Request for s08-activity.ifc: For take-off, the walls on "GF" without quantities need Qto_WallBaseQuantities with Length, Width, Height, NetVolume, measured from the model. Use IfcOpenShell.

First a look at what the model holds.

```python
import ifcopenshell
import ifcopenshell.util.element
import ifcopenshell.util.unit

model = ifcopenshell.open("s08-activity.ifc")
print(model.schema)
for unit_type in ("LENGTHUNIT", "AREAUNIT", "VOLUMEUNIT"):
    print(unit_type, ifcopenshell.util.unit.calculate_unit_scale(model, unit_type))
storey = next(s for s in model.by_type("IfcBuildingStorey") if s.Name == "GF")
walls = [e for e in ifcopenshell.util.element.get_decomposition(storey) if e.is_a("IfcWall")]
for e in sorted(walls, key=lambda e: e.id()):
    print(e.id(), e.is_a(), e.Name, list(ifcopenshell.util.element.get_psets(e, qtos_only=True)), sep=" | ")
```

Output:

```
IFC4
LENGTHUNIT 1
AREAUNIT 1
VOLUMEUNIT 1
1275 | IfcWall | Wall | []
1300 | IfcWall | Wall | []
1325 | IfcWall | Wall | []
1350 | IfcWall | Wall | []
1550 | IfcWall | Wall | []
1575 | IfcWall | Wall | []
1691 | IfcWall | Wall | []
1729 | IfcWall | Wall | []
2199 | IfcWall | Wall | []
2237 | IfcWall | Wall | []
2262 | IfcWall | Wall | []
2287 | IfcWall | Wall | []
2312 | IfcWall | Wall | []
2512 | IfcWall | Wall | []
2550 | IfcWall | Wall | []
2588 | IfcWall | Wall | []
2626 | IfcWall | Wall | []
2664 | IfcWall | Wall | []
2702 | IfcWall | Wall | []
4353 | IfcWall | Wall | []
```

```python
import ifcopenshell
import ifcopenshell.api.pset
import ifcopenshell.geom
import ifcopenshell.util.element
import ifcopenshell.util.shape
import ifcopenshell.util.unit

model = ifcopenshell.open("s08-activity.ifc")
unit_scale = ifcopenshell.util.unit.calculate_unit_scale(model)
volume_scale = ifcopenshell.util.unit.calculate_unit_scale(model, "VOLUMEUNIT")
settings = ifcopenshell.geom.settings()

storey = next(s for s in model.by_type("IfcBuildingStorey") if s.Name == "GF")
walls = [e for e in ifcopenshell.util.element.get_decomposition(storey) if e.is_a("IfcWall")]

for e in sorted(walls, key=lambda e: e.id()):
    if ifcopenshell.util.element.get_psets(e, qtos_only=True, should_inherit=False):
        continue
    # Geometry comes back in metres, in the element's own axes.
    shape = ifcopenshell.geom.create_shape(settings, e)
    values = {
        "Length": ifcopenshell.util.shape.get_x(shape.geometry) / unit_scale,
        "Width": ifcopenshell.util.shape.get_y(shape.geometry) / unit_scale,
        "Height": ifcopenshell.util.shape.get_z(shape.geometry) / unit_scale,
        "NetVolume": ifcopenshell.util.shape.get_volume(shape.geometry) / volume_scale,
    }
    qto = ifcopenshell.api.pset.add_qto(model, product=e, name="Qto_WallBaseQuantities")
    ifcopenshell.api.pset.edit_qto(model, qto=qto, properties=values)
    print(e.id(), {k: round(v, 3) for k, v in values.items()})

model.write("s08-activity_updated.ifc")
```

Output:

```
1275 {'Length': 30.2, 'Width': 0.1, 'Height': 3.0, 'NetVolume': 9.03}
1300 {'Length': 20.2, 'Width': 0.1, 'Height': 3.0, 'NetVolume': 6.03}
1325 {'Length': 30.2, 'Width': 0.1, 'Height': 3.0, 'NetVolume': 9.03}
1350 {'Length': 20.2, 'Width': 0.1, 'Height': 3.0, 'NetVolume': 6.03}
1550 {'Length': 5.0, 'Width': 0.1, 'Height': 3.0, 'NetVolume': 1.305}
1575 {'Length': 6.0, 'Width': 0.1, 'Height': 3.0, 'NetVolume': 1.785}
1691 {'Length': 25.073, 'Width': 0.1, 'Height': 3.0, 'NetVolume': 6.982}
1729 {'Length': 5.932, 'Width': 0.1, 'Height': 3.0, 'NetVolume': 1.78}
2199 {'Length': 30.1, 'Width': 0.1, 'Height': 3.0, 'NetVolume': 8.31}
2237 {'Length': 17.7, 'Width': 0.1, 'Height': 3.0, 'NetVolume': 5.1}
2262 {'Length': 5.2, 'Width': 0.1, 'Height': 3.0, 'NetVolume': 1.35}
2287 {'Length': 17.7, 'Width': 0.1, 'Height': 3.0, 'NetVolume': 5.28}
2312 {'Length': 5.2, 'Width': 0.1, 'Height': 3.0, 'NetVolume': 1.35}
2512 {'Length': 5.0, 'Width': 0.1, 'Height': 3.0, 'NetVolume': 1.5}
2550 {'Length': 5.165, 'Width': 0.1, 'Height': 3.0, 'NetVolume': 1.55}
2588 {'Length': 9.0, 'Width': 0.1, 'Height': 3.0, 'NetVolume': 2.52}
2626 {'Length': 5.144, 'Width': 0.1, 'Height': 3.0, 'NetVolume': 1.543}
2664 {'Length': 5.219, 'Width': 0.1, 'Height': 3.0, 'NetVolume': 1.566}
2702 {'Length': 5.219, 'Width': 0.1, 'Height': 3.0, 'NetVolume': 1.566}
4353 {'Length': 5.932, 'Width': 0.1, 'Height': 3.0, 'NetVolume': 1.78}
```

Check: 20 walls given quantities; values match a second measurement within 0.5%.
